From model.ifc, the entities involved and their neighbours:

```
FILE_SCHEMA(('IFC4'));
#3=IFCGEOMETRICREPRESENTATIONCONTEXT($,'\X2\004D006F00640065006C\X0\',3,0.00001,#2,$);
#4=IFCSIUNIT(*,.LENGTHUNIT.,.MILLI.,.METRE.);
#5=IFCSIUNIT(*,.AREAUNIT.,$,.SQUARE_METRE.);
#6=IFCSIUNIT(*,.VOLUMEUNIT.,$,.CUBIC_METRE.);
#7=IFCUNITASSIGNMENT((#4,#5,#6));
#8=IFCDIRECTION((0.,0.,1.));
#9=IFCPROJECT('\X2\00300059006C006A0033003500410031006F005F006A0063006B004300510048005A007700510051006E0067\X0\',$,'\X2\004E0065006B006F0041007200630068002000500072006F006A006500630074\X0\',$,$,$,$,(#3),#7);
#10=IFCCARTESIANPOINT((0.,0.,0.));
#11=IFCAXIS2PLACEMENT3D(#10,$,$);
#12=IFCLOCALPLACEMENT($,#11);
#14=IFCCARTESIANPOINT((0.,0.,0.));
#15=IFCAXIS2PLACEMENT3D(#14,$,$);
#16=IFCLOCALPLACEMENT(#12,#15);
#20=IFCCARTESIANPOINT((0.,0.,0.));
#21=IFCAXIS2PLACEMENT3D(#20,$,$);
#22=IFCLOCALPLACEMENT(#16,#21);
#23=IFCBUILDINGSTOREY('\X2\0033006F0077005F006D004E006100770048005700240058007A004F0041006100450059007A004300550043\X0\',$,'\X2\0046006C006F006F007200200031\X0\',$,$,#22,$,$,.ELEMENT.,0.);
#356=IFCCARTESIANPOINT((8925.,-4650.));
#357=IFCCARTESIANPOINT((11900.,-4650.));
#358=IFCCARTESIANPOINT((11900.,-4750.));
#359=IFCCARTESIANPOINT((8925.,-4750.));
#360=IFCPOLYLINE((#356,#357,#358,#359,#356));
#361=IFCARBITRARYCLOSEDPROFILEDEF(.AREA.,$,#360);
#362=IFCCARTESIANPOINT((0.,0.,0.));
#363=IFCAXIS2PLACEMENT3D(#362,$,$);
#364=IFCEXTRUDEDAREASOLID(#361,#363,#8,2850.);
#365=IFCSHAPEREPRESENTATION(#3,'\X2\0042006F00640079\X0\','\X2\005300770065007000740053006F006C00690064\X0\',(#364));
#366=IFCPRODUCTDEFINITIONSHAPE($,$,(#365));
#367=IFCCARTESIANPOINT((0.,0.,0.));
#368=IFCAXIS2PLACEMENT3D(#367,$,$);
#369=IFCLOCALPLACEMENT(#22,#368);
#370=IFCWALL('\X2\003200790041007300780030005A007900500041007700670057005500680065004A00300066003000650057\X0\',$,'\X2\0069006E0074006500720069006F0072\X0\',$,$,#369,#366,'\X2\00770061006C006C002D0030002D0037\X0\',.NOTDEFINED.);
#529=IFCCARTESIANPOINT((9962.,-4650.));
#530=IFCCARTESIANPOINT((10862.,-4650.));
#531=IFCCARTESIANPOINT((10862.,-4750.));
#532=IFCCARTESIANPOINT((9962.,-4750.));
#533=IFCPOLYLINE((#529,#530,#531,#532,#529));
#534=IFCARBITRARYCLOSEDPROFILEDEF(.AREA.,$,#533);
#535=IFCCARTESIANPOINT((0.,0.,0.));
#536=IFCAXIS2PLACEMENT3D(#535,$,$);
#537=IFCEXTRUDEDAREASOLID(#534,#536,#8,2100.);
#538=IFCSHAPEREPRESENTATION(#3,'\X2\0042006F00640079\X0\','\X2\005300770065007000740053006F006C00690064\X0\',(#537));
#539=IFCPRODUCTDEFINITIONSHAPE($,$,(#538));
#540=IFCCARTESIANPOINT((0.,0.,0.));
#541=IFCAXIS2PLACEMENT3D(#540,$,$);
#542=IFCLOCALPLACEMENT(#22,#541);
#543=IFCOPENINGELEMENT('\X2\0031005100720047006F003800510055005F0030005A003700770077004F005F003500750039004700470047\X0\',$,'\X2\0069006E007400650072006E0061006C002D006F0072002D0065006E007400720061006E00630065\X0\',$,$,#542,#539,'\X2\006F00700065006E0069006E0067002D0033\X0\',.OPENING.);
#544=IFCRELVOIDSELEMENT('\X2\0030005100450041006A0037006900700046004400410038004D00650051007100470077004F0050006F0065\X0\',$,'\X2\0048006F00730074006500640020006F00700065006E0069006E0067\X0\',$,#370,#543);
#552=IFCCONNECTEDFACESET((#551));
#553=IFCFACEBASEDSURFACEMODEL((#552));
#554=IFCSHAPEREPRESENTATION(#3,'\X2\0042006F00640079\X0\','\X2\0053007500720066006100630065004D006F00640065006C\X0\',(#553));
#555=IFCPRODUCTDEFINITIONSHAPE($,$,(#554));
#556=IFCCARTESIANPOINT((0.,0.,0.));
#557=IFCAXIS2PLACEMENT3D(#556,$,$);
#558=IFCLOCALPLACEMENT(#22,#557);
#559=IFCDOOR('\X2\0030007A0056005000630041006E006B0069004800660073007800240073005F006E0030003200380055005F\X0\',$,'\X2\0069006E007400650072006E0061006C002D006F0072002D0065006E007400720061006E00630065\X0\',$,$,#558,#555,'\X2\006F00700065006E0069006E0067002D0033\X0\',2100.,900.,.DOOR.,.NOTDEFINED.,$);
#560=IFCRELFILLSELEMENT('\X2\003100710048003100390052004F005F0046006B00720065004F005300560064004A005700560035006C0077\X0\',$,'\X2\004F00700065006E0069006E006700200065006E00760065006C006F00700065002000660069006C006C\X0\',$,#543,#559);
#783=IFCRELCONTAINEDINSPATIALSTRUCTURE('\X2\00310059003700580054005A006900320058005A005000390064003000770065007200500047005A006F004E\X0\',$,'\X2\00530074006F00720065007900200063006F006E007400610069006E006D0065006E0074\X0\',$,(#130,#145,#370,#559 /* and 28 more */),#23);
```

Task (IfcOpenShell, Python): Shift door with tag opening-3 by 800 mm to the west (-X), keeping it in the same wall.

```python
import ifcopenshell
import ifcopenshell.api.geometry
import ifcopenshell.util.placement

model = ifcopenshell.open("model.ifc")

door = model.by_guid("0zVPcAnkiHfsx$s_n028U_")
opening = door.FillsVoids[0].RelatingOpeningElement
wall = opening.VoidsElements[0].RelatingBuildingElement

wall_matrix = ifcopenshell.util.placement.get_local_placement(wall.ObjectPlacement)
shift = wall_matrix[:3, 0] * -800.0
before = ifcopenshell.util.placement.get_local_placement(door.ObjectPlacement)[:3, 3].copy()

# The door is not placed relative to its opening, so move both.
for product in (opening, door):
    matrix = ifcopenshell.util.placement.get_local_placement(product.ObjectPlacement)
    matrix[:3, 3] += shift
    ifcopenshell.api.geometry.edit_object_placement(model, product=product, matrix=matrix, is_si=False)

after = ifcopenshell.util.placement.get_local_placement(door.ObjectPlacement)[:3, 3]
print("door moved by", (after - before).round(3) + 0.0)

model.write("model_rev.ifc")
```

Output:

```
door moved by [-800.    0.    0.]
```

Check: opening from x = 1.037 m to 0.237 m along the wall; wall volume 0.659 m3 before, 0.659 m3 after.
